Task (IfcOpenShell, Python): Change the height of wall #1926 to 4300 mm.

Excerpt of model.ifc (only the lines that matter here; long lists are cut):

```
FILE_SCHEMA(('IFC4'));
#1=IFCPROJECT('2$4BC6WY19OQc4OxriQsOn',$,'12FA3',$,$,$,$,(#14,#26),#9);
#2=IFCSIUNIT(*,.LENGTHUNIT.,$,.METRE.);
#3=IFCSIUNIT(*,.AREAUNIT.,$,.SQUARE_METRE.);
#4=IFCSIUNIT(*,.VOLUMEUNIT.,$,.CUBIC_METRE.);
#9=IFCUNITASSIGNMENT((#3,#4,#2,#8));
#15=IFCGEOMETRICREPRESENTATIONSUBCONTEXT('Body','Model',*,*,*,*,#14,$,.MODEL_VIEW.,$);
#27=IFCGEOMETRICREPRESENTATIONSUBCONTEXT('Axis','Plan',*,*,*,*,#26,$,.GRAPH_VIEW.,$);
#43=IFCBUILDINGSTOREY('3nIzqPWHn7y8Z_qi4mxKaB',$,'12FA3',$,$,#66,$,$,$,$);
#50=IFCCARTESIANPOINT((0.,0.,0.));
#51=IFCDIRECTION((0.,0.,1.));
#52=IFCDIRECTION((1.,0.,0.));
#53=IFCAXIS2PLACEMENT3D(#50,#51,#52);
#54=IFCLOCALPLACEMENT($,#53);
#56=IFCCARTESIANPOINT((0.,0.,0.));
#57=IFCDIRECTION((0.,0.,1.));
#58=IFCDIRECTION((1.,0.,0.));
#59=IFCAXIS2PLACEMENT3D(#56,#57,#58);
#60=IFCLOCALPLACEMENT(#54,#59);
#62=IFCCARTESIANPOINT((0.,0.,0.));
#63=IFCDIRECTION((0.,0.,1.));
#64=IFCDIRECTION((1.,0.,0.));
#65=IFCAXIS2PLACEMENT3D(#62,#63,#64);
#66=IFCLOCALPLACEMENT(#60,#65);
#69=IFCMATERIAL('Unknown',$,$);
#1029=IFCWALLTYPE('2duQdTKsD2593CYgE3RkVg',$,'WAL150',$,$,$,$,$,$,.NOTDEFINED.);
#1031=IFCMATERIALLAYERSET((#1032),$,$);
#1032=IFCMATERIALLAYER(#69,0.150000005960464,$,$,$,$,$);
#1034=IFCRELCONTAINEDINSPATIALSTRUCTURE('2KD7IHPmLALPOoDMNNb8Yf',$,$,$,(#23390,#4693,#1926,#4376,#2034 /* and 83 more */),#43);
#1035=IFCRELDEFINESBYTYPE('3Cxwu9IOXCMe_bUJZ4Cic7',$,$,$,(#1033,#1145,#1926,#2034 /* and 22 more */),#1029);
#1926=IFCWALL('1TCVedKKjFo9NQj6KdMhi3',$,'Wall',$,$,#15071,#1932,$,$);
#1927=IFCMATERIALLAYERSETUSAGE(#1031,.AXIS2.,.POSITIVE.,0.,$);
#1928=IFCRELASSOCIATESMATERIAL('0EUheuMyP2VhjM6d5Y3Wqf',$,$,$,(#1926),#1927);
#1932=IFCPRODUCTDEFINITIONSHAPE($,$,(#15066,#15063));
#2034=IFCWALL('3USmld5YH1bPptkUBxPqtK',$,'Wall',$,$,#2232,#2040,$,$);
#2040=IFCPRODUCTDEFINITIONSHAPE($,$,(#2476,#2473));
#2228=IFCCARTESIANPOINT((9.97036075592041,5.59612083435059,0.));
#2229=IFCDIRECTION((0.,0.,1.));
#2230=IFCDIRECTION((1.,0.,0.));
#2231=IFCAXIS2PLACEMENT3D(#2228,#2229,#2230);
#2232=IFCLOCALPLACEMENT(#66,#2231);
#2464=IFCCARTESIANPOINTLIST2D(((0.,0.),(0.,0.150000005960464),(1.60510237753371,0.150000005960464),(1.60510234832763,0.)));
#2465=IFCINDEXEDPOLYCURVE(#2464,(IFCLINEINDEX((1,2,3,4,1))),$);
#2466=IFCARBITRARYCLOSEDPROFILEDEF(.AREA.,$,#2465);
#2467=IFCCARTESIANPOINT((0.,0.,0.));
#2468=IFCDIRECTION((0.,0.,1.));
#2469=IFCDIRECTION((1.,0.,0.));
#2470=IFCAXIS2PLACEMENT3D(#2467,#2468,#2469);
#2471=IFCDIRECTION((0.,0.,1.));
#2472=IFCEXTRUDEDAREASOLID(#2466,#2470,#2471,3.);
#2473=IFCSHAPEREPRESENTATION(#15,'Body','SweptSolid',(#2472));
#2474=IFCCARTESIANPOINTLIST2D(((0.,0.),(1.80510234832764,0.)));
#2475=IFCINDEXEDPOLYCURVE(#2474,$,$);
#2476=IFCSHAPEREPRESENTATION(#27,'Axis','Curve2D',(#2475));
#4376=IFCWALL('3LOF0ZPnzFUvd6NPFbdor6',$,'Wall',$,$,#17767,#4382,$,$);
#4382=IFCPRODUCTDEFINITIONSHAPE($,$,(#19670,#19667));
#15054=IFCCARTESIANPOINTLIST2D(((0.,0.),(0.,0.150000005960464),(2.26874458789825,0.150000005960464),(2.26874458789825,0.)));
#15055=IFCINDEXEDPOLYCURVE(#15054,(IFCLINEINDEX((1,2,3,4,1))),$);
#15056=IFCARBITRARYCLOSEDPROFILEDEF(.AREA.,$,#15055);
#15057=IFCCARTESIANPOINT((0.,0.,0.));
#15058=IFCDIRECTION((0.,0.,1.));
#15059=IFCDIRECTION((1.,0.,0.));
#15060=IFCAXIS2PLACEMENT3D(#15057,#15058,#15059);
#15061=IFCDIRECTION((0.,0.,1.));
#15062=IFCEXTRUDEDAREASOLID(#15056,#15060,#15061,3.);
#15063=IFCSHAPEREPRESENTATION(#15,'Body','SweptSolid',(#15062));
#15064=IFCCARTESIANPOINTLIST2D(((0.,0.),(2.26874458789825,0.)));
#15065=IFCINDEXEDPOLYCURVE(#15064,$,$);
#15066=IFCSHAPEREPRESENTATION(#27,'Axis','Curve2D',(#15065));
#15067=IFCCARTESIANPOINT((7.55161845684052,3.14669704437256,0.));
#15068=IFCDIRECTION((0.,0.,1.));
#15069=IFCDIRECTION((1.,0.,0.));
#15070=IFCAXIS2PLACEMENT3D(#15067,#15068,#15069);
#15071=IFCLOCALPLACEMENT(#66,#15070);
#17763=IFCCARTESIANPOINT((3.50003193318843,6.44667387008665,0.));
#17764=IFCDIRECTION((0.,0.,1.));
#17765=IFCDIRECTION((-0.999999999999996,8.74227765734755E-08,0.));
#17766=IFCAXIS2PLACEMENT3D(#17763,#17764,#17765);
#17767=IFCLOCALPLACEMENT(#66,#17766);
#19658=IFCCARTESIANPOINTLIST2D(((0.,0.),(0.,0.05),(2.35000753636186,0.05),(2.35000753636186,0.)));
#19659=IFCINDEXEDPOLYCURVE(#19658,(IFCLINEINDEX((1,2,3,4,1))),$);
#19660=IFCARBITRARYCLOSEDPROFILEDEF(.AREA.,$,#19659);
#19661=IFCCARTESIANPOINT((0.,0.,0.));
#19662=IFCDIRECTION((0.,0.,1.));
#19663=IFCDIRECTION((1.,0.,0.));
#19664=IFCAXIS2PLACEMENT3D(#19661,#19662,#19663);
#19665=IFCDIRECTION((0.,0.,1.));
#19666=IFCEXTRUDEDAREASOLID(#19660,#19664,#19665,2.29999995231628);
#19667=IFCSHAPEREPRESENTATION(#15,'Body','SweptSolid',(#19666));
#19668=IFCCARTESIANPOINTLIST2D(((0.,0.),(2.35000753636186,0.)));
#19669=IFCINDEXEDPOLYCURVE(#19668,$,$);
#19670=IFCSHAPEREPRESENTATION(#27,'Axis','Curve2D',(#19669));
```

```python
import ifcopenshell
import ifcopenshell.geom
import ifcopenshell.util.representation
import ifcopenshell.util.shape
import ifcopenshell.util.unit

model = ifcopenshell.open("model.ifc")
unit_scale = ifcopenshell.util.unit.calculate_unit_scale(model)
settings = ifcopenshell.geom.settings()


def volume(element):
    """Net volume in cubic metres, openings subtracted."""
    shape = ifcopenshell.geom.create_shape(settings, element)
    return ifcopenshell.util.shape.get_volume(shape.geometry)


wall = model.by_guid("1TCVedKKjFo9NQj6KdMhi3")
before = volume(wall)

body = ifcopenshell.util.representation.get_representation(wall, "Model", "Body")
solid = body.Items[0]
old_height = solid.Depth
solid.Depth = 4.3 / unit_scale
after = volume(wall)

print(f"height {old_height:g} -> {solid.Depth:g}, volume {before:.3f} -> {after:.3f} m3")

model.write("model-out.ifc")
```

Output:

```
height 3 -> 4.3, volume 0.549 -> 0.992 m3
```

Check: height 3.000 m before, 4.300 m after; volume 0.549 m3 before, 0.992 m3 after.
